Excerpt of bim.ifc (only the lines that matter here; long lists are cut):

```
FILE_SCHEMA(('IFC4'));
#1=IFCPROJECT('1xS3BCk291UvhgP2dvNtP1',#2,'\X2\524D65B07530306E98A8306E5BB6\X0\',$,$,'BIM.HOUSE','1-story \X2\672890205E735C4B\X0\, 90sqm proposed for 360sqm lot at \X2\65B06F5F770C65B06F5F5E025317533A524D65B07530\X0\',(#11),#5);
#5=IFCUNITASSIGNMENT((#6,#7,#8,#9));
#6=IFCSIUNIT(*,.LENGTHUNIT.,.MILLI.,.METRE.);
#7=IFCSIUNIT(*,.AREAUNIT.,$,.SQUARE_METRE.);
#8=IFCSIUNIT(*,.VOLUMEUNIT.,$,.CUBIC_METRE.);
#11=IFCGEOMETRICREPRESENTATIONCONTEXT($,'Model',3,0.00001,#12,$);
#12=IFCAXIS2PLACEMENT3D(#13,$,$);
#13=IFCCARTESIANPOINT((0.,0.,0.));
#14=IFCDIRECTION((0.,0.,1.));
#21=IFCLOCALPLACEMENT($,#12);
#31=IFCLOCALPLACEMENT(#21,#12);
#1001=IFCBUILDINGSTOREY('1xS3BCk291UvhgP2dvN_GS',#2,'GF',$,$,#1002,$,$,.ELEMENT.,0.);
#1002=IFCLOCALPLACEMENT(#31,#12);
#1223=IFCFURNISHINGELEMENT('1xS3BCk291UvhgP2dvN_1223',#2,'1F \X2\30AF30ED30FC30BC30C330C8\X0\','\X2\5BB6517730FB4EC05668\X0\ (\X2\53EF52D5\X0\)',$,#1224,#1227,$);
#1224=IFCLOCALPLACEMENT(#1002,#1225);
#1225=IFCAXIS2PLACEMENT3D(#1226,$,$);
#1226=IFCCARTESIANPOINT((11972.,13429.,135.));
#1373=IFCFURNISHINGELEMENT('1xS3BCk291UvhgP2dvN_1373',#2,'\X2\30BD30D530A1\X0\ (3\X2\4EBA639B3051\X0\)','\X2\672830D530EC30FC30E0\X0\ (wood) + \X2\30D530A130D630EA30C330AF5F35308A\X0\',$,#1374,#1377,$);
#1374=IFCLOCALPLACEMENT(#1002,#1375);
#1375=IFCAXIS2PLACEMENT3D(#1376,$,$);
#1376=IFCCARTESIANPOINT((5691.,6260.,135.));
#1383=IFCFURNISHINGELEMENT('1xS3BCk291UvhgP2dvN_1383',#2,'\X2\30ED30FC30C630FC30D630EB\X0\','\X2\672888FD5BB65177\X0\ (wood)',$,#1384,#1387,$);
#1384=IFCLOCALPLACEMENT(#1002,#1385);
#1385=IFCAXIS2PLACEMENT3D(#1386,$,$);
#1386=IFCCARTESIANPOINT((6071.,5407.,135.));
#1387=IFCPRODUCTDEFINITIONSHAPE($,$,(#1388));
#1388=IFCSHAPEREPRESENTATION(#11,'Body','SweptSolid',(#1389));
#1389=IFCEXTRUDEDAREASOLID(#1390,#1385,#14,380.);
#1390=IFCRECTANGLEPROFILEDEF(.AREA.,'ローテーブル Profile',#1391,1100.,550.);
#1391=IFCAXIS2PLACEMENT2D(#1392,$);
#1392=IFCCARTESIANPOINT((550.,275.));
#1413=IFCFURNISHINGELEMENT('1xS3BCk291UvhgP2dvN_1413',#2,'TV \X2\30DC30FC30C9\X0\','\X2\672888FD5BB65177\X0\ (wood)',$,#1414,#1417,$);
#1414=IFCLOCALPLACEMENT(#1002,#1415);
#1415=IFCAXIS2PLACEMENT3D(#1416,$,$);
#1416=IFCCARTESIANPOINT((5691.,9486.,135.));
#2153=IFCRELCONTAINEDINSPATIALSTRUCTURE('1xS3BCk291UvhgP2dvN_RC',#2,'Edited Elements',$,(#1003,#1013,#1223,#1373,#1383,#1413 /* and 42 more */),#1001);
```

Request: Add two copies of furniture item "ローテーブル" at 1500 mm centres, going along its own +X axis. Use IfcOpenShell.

```python
import ifcopenshell
import ifcopenshell.api.geometry
import ifcopenshell.api.root
import ifcopenshell.util.element
import ifcopenshell.util.placement
import ifcopenshell.util.unit

model = ifcopenshell.open("bim.ifc")
unit_scale = ifcopenshell.util.unit.calculate_unit_scale(model)


def reuse_history(source, copy):
    """copy_class also copies each property set's owner history, people and application; keep the originals."""
    for rel in copy.IsDefinedBy:
        if rel.is_a("IfcRelDefinesByProperties") and (history := rel.RelatingPropertyDefinition.OwnerHistory):
            rel.RelatingPropertyDefinition.OwnerHistory = source.OwnerHistory
            ifcopenshell.util.element.remove_deep2(model, history)


source = model.by_guid("1xS3BCk291UvhgP2dvN_1383")
base = ifcopenshell.util.placement.get_local_placement(source.ObjectPlacement)
step = base[:3, 0] * 1.5 / unit_scale

for i in range(1, 3):
    copy = ifcopenshell.api.root.copy_class(model, product=source)
    copy.Representation = ifcopenshell.util.element.copy_deep(
        model, source.Representation, exclude=["IfcGeometricRepresentationContext", "IfcRepresentationMap"]
    )
    reuse_history(source, copy)
    matrix = base.copy()
    matrix[:3, 3] += i * step
    print("added at", matrix[:3, 3].round(3) + 0.0)
    ifcopenshell.api.geometry.edit_object_placement(model, product=copy, matrix=matrix, is_si=False)

model.write("bim_updated.ifc")
```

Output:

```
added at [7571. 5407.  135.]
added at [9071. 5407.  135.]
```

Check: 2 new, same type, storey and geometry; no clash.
